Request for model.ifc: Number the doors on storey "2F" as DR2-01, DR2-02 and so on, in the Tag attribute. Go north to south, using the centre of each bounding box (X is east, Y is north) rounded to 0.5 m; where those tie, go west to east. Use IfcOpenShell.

First a look at what the model holds.

```python
import ifcopenshell
import ifcopenshell.util.element
import ifcopenshell.util.placement

model = ifcopenshell.open("model.ifc")
print(model.schema)
storey = next(s for s in model.by_type("IfcBuildingStorey") if s.Name == "2F")
doors = [e for e in ifcopenshell.util.element.get_decomposition(storey) if e.is_a("IfcDoor")]
for e in sorted(doors, key=lambda e: e.id()):
    origin = ifcopenshell.util.placement.get_local_placement(e.ObjectPlacement)[:3, 3]
    print(e.id(), e.Tag, e.Name, origin.round(2) + 0.0, sep=" | ")
```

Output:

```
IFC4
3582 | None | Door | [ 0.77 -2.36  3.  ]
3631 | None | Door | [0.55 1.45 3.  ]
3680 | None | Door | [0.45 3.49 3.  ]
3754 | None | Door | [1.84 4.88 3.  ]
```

```python
import ifcopenshell
import ifcopenshell.geom
import ifcopenshell.util.element
import ifcopenshell.util.shape

model = ifcopenshell.open("model.ifc")
settings = ifcopenshell.geom.settings()
settings.set("use-world-coords", True)


def centre(element):
    shape = ifcopenshell.geom.create_shape(settings, element)
    return ifcopenshell.util.shape.get_bbox_centroid(shape.geometry)


storey = next(s for s in model.by_type("IfcBuildingStorey") if s.Name == "2F")
doors = [e for e in ifcopenshell.util.element.get_decomposition(storey) if e.is_a("IfcDoor")]

# Insertion points can sit at a corner or the storey origin, so sort by the geometry (in metres).
centres = {e: centre(e) for e in doors}
doors.sort(key=lambda e: (-round(centres[e][1] / 0.5), centres[e][0]))

for i, e in enumerate(doors, start=1):
    number = f"DR2-{i:02d}"
    e.Tag = number
    print(e.id(), number)

model.write("model_rev.ifc")
```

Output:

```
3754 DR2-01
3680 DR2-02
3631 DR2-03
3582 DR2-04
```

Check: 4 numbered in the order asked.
